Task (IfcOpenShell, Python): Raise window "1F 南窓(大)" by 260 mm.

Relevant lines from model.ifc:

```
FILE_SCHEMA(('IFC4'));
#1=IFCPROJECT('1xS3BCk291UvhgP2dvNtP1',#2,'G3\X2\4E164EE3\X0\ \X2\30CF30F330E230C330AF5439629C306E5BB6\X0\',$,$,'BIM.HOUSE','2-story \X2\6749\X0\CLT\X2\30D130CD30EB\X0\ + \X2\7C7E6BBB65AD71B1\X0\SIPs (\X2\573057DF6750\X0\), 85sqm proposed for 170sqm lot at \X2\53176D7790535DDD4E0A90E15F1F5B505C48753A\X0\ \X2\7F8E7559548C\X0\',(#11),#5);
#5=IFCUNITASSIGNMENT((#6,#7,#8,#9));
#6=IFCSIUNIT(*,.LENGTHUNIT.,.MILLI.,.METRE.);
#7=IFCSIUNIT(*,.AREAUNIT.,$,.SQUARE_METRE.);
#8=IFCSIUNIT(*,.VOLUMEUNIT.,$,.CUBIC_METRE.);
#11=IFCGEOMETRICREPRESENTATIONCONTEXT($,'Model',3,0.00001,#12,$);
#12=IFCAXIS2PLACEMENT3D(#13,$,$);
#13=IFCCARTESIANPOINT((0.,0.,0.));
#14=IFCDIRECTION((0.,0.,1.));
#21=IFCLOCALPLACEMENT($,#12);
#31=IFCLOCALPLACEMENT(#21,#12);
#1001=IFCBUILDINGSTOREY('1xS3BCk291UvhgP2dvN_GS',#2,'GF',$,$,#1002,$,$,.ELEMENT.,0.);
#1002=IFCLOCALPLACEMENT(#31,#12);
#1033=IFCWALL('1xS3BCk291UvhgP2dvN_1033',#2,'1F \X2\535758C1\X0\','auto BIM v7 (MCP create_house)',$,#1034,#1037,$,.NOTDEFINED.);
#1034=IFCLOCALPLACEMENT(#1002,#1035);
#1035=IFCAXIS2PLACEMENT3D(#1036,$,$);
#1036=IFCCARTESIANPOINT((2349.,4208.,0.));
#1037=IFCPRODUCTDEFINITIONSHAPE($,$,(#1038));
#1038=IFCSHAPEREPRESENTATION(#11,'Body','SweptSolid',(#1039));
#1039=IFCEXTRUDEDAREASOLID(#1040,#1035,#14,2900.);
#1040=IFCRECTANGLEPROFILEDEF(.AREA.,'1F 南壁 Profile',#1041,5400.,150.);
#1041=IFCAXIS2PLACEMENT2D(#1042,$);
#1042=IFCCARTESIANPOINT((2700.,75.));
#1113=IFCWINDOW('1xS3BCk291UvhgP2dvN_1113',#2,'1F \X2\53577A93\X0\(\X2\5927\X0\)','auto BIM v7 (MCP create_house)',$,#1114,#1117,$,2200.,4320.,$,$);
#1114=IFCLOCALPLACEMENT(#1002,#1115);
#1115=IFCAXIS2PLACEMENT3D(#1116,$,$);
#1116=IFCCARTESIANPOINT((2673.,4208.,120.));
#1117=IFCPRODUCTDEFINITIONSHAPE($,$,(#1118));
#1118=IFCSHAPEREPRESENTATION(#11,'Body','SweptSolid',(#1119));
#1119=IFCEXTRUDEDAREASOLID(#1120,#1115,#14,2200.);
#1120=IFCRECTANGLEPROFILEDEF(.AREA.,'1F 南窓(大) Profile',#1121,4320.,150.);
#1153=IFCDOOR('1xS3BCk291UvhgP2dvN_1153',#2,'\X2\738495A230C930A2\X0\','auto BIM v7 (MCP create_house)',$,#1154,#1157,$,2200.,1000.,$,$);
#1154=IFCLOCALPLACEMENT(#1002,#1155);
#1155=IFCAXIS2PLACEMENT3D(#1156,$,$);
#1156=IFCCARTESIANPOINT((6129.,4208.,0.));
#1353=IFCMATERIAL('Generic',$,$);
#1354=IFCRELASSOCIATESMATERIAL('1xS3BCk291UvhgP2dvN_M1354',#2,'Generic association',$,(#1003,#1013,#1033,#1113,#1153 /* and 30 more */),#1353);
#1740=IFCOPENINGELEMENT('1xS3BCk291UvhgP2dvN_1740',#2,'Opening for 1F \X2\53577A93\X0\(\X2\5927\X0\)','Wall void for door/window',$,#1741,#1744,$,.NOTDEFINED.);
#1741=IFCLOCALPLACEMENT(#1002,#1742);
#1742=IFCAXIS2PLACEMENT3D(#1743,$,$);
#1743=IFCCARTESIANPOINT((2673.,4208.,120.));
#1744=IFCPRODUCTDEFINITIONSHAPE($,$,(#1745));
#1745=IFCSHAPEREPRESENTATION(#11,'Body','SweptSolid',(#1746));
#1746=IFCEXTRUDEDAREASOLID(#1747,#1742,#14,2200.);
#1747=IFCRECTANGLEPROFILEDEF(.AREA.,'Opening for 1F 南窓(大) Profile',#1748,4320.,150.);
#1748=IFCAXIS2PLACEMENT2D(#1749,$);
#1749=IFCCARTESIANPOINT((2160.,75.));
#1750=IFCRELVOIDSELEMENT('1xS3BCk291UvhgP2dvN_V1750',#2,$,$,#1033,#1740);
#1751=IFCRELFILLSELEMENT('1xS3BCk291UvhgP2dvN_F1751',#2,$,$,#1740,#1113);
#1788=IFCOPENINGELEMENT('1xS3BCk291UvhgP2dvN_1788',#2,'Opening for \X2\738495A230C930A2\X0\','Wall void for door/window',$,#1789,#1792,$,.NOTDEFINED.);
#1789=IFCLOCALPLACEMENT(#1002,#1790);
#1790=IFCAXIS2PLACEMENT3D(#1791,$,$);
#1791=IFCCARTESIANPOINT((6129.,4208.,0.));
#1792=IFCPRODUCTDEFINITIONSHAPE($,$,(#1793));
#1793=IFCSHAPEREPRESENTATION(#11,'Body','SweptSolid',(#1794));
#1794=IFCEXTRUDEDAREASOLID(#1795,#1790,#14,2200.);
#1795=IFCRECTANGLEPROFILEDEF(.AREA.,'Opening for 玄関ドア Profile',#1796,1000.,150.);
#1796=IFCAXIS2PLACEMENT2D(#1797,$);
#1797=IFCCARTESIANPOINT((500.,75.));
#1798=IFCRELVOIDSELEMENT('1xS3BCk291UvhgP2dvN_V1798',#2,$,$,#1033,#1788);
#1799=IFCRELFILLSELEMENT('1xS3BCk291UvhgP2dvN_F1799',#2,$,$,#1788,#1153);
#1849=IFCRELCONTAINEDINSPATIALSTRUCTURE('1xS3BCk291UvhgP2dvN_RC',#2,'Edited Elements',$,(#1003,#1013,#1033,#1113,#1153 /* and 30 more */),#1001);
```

```python
import numpy as np
import ifcopenshell
import ifcopenshell.api.geometry
import ifcopenshell.util.placement
import ifcopenshell.util.unit

model = ifcopenshell.open("model.ifc")
unit_scale = ifcopenshell.util.unit.calculate_unit_scale(model)

window = model.by_guid("1xS3BCk291UvhgP2dvN_1113")
opening = window.FillsVoids[0].RelatingOpeningElement
dz = 260.0

shift = np.array([0.0, 0.0, dz])
# The window is not placed relative to its opening, so move both.
for product in (opening, window):
    matrix = ifcopenshell.util.placement.get_local_placement(product.ObjectPlacement)
    matrix[:3, 3] += shift
    ifcopenshell.api.geometry.edit_object_placement(model, product=product, matrix=matrix, is_si=False)

print(f"moved by {dz * unit_scale:+.3f} m")

model.write("model_updated.ifc")
```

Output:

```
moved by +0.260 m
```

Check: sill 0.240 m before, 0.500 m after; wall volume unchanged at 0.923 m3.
